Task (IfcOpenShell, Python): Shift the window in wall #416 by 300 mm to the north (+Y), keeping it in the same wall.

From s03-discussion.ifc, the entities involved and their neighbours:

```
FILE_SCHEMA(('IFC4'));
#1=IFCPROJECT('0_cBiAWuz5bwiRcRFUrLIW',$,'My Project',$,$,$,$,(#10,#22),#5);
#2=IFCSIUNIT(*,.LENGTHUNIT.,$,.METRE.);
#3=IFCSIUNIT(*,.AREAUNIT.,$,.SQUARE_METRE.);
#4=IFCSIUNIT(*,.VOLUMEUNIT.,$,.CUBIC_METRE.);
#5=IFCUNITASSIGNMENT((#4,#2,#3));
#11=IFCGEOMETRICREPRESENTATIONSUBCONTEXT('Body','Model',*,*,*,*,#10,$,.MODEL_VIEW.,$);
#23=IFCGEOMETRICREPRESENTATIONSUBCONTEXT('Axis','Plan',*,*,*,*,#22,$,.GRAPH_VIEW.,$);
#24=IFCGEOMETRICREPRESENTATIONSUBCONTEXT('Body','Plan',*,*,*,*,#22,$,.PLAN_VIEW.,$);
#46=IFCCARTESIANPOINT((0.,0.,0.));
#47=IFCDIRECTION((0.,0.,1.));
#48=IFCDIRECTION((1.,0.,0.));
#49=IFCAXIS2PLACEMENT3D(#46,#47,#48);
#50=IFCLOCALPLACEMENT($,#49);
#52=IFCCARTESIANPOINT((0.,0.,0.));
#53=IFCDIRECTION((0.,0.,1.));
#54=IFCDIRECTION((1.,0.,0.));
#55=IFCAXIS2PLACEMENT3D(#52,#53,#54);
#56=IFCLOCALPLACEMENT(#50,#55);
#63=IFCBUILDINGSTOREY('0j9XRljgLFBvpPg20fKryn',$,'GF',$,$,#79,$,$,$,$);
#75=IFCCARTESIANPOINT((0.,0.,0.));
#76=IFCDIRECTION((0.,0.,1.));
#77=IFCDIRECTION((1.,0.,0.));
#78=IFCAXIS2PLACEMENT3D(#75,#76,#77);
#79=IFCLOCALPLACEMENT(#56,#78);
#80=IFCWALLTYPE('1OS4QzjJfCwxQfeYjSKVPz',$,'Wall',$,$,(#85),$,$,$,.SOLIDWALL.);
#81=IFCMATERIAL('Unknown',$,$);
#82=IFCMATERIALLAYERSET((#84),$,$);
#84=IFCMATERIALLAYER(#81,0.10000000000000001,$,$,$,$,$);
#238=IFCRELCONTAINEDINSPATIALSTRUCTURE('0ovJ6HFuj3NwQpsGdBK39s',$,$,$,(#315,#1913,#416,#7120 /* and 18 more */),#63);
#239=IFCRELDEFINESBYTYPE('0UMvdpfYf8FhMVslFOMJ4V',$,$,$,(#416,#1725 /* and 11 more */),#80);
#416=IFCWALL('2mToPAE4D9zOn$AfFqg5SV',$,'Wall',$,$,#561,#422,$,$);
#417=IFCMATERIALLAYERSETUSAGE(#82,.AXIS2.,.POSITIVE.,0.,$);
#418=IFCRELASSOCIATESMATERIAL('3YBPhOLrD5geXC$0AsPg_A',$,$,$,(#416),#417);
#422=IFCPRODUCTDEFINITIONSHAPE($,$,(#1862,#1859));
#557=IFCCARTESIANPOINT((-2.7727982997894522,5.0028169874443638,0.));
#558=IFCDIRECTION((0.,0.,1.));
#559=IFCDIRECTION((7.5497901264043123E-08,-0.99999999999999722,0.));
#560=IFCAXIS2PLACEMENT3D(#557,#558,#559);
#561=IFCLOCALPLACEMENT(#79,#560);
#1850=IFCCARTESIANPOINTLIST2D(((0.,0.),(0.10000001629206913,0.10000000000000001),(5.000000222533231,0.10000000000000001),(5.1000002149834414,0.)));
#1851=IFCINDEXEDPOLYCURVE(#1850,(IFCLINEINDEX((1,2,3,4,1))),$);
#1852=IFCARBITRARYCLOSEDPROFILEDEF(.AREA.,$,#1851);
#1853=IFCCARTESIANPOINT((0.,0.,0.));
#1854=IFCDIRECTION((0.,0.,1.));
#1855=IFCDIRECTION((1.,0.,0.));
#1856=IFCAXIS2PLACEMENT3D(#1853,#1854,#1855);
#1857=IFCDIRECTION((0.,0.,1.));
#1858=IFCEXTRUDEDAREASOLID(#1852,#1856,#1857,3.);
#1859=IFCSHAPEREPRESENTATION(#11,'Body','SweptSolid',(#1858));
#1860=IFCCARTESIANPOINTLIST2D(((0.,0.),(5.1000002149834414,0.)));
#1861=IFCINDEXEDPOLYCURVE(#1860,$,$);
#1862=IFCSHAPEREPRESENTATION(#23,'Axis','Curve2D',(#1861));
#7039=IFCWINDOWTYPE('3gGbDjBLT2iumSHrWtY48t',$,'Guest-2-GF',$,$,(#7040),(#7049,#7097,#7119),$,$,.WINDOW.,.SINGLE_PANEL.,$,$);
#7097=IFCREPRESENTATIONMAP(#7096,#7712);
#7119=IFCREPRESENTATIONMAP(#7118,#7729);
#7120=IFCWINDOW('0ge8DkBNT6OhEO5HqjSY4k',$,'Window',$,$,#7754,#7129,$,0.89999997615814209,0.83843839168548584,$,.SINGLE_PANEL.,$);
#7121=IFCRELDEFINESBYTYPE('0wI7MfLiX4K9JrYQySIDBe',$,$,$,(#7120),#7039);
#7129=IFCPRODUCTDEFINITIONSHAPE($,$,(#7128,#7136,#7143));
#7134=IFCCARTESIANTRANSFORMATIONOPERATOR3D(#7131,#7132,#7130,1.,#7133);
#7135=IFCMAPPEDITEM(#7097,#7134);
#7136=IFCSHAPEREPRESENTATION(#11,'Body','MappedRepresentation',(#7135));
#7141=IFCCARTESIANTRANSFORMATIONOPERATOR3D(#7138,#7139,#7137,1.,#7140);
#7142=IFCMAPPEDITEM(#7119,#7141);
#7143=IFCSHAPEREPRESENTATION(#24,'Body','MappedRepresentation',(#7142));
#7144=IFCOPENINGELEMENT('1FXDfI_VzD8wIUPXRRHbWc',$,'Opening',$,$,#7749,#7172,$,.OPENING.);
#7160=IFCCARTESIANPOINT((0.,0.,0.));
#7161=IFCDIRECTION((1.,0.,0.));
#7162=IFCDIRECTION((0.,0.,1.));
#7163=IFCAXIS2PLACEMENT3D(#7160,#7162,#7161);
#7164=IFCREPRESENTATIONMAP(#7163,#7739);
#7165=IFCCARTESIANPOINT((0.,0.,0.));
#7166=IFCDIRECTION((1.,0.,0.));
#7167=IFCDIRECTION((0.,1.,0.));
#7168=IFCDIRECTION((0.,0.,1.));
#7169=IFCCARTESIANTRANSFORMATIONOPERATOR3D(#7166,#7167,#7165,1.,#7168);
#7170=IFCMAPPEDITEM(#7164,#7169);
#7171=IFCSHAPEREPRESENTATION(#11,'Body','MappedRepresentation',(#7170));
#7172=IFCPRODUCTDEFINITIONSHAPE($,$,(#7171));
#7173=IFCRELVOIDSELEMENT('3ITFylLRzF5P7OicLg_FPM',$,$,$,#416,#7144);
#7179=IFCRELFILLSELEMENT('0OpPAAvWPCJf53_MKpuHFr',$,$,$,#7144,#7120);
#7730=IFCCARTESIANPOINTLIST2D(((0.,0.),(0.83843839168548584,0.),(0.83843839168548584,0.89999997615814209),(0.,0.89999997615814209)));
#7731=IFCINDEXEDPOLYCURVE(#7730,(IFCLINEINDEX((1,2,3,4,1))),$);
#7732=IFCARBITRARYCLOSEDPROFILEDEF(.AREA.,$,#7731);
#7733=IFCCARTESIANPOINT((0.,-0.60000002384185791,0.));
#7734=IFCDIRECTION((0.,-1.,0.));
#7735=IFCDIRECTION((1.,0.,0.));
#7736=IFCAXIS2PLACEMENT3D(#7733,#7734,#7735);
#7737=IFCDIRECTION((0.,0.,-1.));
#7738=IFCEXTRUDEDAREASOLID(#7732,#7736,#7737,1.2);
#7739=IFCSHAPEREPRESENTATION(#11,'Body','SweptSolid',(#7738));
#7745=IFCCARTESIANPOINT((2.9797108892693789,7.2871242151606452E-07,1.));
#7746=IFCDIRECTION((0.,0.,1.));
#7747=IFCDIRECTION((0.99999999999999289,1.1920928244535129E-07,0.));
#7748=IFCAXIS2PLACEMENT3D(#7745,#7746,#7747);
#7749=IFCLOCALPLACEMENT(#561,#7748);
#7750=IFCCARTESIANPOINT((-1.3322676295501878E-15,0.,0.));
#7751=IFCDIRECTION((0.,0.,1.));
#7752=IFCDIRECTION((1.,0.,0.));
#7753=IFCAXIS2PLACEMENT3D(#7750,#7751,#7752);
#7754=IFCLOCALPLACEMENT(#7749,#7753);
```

```python
import ifcopenshell
import ifcopenshell.api.geometry
import ifcopenshell.util.placement
import ifcopenshell.util.unit

model = ifcopenshell.open("s03-discussion.ifc")
unit_scale = ifcopenshell.util.unit.calculate_unit_scale(model)

window = model.by_guid("0ge8DkBNT6OhEO5HqjSY4k")
opening = window.FillsVoids[0].RelatingOpeningElement
wall = opening.VoidsElements[0].RelatingBuildingElement

wall_matrix = ifcopenshell.util.placement.get_local_placement(wall.ObjectPlacement)
shift = wall_matrix[:3, 0] * -0.3 / unit_scale
before = ifcopenshell.util.placement.get_local_placement(window.ObjectPlacement)[:3, 3].copy()

# The window is placed relative to its opening, so it follows when the opening moves.
matrix = ifcopenshell.util.placement.get_local_placement(opening.ObjectPlacement)
matrix[:3, 3] += shift
ifcopenshell.api.geometry.edit_object_placement(
    model, product=opening, matrix=matrix, is_si=False, should_transform_children=True
)

after = ifcopenshell.util.placement.get_local_placement(window.ObjectPlacement)[:3, 3]
print("window moved by", (after - before).round(3) + 0.0)

model.write("s03-discussion_rev.ifc")
```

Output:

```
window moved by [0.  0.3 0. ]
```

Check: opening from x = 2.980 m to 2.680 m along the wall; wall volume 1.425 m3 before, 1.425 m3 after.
